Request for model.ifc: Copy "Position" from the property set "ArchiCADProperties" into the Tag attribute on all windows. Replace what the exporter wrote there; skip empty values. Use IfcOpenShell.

First a look at what the model holds.

```python
import ifcopenshell
import ifcopenshell.util.element

model = ifcopenshell.open("model.ifc")
print(model.schema)
windows = model.by_type("IfcWindow")
print(len(windows), "windows")
for e in windows[:8]:
    source = ifcopenshell.util.element.get_pset(e, "ArchiCADProperties", "Position")
    target = e.Tag
    print(e.id(), repr(source), repr(target), sep=" | ")
```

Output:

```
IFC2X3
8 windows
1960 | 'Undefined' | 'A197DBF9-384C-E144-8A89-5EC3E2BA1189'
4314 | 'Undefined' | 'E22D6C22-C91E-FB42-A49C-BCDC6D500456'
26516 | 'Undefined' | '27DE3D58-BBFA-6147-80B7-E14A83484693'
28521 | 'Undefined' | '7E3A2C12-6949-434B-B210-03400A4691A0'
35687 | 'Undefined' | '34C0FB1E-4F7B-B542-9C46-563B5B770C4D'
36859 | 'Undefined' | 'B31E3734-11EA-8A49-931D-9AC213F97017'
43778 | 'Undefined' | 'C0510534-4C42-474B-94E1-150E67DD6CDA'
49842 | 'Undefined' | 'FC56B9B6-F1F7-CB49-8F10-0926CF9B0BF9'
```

```python
import ifcopenshell
import ifcopenshell.util.element

model = ifcopenshell.open("model.ifc")

count = 0
for e in model.by_type("IfcWindow"):
    value = ifcopenshell.util.element.get_pset(e, "ArchiCADProperties", "Position")
    current = e.Tag
    if not value or not value.strip() or current == value:
        continue
    e.Tag = value
    count += 1

print(count, "windows updated")

model.write("model_v2.ifc")
```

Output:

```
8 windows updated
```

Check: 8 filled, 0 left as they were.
